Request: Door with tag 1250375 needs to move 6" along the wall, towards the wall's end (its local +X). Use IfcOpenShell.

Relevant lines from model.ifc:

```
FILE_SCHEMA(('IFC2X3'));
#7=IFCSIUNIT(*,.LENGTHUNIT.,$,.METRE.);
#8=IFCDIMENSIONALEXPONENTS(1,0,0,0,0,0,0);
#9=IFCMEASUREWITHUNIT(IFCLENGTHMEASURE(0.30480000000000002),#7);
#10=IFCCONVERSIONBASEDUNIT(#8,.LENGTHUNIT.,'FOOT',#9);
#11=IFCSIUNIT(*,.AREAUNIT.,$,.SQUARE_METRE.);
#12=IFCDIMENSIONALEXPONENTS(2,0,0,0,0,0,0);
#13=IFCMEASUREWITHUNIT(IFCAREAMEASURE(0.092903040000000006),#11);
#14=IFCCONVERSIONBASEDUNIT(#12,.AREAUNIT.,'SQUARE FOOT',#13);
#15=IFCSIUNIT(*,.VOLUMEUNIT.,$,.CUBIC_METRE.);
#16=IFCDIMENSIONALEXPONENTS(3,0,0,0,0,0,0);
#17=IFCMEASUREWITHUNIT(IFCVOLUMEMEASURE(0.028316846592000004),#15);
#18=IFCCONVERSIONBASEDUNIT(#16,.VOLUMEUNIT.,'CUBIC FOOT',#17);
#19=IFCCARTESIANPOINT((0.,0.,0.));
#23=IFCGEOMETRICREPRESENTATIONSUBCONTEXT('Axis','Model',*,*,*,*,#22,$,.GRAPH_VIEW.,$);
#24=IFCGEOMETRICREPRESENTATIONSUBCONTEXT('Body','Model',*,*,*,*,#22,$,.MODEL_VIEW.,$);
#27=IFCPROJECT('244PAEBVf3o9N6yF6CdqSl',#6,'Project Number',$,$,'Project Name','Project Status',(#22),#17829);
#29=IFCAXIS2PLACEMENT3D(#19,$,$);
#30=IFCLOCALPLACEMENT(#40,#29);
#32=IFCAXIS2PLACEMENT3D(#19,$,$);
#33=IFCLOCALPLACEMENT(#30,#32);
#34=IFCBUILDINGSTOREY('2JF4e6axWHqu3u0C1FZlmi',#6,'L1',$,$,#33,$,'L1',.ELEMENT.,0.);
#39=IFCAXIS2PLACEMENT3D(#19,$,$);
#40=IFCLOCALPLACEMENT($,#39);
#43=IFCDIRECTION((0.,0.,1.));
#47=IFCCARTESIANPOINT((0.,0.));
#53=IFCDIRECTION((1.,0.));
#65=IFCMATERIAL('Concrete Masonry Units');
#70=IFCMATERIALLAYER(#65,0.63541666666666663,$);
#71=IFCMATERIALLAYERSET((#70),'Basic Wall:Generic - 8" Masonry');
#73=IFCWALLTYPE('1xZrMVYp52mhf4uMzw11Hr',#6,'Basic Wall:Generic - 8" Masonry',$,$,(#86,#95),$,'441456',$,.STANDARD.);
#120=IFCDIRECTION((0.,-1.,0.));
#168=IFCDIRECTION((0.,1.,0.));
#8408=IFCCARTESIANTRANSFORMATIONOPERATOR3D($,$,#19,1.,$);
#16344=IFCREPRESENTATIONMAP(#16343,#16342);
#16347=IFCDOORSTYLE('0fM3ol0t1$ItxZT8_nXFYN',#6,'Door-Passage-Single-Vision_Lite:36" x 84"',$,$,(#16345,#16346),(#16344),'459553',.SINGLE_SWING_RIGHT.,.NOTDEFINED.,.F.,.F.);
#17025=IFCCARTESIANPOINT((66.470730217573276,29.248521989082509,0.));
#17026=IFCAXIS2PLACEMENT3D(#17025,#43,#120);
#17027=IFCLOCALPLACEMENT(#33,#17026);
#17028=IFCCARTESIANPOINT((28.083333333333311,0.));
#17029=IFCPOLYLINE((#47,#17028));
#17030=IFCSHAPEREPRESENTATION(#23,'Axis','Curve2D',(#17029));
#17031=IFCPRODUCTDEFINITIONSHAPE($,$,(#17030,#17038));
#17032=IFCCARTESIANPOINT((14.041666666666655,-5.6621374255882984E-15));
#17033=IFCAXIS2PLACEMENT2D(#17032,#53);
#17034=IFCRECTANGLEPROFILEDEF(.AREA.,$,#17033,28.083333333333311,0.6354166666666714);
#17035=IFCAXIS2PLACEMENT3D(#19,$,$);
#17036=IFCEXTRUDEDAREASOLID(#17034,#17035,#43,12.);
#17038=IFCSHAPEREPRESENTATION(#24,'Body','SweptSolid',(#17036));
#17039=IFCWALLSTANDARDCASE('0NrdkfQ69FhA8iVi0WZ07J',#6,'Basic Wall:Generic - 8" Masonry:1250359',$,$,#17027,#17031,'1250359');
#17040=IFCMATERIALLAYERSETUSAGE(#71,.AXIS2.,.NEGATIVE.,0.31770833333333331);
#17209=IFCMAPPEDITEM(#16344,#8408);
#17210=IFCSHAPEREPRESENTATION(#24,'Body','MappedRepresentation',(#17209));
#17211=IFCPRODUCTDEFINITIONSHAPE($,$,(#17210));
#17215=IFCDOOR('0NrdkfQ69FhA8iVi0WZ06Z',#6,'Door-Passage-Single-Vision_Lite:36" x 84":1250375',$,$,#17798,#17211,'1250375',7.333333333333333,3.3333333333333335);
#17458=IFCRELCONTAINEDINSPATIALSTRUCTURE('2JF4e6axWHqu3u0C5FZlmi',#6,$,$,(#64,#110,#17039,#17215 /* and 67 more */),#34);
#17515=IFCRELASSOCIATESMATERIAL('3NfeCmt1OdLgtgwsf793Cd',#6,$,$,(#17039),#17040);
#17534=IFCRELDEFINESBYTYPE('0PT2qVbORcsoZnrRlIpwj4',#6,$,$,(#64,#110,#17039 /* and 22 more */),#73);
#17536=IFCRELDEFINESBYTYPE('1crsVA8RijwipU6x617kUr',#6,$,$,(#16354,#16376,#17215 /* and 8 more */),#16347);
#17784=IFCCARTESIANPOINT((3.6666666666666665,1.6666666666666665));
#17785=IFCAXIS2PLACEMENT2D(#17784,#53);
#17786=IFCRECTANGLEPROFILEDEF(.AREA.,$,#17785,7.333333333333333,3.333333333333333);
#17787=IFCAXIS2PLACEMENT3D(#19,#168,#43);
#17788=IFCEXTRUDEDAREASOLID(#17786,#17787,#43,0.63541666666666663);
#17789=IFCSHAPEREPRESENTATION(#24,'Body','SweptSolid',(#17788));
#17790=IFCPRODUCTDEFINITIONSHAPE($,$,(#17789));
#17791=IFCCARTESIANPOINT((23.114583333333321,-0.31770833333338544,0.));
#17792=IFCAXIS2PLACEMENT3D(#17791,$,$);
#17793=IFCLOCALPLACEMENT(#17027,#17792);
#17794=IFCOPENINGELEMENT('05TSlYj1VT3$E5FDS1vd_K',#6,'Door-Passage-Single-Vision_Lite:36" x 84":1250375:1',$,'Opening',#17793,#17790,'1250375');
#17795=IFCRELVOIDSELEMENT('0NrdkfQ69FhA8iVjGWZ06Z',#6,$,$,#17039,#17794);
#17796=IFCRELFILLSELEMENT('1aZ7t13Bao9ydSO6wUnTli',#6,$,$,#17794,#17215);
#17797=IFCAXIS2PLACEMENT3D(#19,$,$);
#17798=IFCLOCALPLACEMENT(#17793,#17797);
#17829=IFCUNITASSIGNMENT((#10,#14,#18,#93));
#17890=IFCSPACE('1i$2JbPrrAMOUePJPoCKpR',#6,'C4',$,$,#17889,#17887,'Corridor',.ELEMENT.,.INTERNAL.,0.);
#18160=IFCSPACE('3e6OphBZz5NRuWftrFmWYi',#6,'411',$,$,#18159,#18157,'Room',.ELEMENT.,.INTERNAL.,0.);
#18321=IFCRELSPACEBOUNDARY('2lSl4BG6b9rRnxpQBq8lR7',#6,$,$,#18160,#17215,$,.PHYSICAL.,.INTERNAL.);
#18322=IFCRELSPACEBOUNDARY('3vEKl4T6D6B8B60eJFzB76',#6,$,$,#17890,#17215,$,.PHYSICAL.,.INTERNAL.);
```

```python
import ifcopenshell
import ifcopenshell.api.geometry
import ifcopenshell.util.placement
import ifcopenshell.util.unit

model = ifcopenshell.open("model.ifc")
unit_scale = ifcopenshell.util.unit.calculate_unit_scale(model)

door = model.by_guid("0NrdkfQ69FhA8iVi0WZ06Z")
opening = door.FillsVoids[0].RelatingOpeningElement
wall = opening.VoidsElements[0].RelatingBuildingElement

wall_matrix = ifcopenshell.util.placement.get_local_placement(wall.ObjectPlacement)
shift = wall_matrix[:3, 0] * 6 * 0.0254 / unit_scale
before = ifcopenshell.util.placement.get_local_placement(door.ObjectPlacement)[:3, 3].copy()

# The door is placed relative to its opening, so it follows when the opening moves.
matrix = ifcopenshell.util.placement.get_local_placement(opening.ObjectPlacement)
matrix[:3, 3] += shift
ifcopenshell.api.geometry.edit_object_placement(
    model, product=opening, matrix=matrix, is_si=False, should_transform_children=True
)

after = ifcopenshell.util.placement.get_local_placement(door.ObjectPlacement)[:3, 3]
print("door moved by", (after - before).round(3) + 0.0)

model.write("model_edited.ifc")
```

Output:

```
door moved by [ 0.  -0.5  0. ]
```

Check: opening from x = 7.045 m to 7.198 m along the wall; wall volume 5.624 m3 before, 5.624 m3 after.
